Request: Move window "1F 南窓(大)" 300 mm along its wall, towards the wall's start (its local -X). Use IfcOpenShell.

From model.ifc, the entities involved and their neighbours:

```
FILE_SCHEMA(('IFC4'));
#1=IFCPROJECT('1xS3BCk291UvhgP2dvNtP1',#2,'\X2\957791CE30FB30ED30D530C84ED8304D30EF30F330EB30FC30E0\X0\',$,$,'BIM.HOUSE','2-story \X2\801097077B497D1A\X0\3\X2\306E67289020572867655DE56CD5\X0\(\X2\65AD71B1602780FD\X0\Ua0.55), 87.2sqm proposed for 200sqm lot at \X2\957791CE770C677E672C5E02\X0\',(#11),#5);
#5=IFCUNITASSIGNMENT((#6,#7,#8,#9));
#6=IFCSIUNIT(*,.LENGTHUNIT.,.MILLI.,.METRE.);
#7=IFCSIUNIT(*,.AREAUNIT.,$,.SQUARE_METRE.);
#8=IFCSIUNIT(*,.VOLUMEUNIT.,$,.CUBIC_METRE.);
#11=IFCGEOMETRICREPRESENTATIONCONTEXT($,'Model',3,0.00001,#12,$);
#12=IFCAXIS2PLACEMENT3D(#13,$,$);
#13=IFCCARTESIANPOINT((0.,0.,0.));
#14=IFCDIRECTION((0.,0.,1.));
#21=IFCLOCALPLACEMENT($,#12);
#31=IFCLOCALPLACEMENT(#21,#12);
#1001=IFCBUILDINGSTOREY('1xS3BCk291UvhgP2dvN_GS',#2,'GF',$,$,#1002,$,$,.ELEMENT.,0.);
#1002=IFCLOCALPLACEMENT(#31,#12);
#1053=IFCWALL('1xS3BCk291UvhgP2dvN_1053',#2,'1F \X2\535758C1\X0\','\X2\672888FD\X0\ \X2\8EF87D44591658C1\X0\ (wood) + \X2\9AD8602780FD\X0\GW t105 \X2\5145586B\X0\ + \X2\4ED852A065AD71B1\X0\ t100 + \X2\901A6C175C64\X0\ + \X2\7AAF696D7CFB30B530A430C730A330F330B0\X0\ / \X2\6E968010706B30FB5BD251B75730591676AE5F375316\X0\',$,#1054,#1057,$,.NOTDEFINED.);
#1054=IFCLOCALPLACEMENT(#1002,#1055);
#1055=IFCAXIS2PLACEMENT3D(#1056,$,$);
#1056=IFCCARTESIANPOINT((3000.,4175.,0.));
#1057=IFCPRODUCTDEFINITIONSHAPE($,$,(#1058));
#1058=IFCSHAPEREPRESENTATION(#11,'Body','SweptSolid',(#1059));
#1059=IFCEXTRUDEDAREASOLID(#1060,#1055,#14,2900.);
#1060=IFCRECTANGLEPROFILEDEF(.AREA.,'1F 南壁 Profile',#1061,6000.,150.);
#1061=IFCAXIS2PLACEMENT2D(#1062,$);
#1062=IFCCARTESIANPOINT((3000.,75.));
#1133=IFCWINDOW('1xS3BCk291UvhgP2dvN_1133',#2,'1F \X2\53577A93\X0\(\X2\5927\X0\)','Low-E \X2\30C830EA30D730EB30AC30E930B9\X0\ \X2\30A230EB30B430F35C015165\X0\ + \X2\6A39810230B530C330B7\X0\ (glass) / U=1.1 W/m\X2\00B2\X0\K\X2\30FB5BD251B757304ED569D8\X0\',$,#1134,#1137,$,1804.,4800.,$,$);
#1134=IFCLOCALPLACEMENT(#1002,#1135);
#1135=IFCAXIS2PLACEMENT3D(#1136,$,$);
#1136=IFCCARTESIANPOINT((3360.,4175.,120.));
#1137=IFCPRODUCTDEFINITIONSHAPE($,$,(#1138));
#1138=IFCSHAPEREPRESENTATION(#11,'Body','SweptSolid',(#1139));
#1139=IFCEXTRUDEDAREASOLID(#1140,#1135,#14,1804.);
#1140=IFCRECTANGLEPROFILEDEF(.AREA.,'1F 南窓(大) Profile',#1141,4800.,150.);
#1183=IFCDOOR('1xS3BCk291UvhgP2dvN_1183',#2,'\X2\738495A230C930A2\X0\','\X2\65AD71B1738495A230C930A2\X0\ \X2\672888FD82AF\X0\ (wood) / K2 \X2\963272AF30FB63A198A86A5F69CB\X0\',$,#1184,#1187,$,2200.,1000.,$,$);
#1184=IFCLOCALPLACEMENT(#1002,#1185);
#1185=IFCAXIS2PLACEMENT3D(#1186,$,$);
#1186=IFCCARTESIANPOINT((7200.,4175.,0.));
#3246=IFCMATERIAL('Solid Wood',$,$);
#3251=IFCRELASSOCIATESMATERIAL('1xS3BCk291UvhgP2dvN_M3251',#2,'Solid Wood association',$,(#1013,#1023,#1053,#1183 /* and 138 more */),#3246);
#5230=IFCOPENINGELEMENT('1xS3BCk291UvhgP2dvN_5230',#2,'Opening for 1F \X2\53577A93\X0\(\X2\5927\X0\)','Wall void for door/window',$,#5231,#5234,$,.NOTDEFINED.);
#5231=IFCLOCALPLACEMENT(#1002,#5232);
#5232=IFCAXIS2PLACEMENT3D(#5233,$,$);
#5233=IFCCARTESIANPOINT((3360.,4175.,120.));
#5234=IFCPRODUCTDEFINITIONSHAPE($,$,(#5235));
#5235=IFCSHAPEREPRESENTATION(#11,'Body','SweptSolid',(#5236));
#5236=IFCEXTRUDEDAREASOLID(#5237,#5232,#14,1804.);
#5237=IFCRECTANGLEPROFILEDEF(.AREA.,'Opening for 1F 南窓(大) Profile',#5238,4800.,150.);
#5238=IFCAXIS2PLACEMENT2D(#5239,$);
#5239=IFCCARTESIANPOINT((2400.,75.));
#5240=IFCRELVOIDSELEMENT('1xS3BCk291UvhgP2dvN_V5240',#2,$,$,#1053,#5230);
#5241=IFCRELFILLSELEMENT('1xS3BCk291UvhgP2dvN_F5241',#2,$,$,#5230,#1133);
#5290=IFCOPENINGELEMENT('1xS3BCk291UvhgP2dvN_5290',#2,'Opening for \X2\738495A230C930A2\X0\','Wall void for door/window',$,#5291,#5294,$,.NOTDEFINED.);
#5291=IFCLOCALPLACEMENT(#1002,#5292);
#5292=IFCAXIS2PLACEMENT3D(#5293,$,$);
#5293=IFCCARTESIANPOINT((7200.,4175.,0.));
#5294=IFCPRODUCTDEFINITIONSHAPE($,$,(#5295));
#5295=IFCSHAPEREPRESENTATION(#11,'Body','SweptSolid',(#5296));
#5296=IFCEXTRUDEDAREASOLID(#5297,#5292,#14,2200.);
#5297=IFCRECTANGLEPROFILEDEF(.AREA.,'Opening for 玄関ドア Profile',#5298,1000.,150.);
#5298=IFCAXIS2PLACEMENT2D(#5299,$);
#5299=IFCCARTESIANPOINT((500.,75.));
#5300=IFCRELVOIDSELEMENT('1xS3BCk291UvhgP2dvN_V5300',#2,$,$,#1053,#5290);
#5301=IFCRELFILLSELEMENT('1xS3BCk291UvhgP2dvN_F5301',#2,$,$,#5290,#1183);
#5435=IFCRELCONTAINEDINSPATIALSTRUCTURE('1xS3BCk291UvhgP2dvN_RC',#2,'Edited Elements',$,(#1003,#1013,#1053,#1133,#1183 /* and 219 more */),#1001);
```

```python
import ifcopenshell
import ifcopenshell.api.geometry
import ifcopenshell.util.placement

model = ifcopenshell.open("model.ifc")

window = model.by_id(1133)
opening = window.FillsVoids[0].RelatingOpeningElement
wall = opening.VoidsElements[0].RelatingBuildingElement

wall_matrix = ifcopenshell.util.placement.get_local_placement(wall.ObjectPlacement)
shift = wall_matrix[:3, 0] * -300.0
before = ifcopenshell.util.placement.get_local_placement(window.ObjectPlacement)[:3, 3].copy()

# The window is not placed relative to its opening, so move both.
for product in (opening, window):
    matrix = ifcopenshell.util.placement.get_local_placement(product.ObjectPlacement)
    matrix[:3, 3] += shift
    ifcopenshell.api.geometry.edit_object_placement(model, product=product, matrix=matrix, is_si=False)

after = ifcopenshell.util.placement.get_local_placement(window.ObjectPlacement)[:3, 3]
print("window moved by", (after - before).round(3) + 0.0)

model.write("model_rev.ifc")
```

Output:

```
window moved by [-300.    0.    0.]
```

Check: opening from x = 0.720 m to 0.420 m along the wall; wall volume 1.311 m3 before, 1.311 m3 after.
